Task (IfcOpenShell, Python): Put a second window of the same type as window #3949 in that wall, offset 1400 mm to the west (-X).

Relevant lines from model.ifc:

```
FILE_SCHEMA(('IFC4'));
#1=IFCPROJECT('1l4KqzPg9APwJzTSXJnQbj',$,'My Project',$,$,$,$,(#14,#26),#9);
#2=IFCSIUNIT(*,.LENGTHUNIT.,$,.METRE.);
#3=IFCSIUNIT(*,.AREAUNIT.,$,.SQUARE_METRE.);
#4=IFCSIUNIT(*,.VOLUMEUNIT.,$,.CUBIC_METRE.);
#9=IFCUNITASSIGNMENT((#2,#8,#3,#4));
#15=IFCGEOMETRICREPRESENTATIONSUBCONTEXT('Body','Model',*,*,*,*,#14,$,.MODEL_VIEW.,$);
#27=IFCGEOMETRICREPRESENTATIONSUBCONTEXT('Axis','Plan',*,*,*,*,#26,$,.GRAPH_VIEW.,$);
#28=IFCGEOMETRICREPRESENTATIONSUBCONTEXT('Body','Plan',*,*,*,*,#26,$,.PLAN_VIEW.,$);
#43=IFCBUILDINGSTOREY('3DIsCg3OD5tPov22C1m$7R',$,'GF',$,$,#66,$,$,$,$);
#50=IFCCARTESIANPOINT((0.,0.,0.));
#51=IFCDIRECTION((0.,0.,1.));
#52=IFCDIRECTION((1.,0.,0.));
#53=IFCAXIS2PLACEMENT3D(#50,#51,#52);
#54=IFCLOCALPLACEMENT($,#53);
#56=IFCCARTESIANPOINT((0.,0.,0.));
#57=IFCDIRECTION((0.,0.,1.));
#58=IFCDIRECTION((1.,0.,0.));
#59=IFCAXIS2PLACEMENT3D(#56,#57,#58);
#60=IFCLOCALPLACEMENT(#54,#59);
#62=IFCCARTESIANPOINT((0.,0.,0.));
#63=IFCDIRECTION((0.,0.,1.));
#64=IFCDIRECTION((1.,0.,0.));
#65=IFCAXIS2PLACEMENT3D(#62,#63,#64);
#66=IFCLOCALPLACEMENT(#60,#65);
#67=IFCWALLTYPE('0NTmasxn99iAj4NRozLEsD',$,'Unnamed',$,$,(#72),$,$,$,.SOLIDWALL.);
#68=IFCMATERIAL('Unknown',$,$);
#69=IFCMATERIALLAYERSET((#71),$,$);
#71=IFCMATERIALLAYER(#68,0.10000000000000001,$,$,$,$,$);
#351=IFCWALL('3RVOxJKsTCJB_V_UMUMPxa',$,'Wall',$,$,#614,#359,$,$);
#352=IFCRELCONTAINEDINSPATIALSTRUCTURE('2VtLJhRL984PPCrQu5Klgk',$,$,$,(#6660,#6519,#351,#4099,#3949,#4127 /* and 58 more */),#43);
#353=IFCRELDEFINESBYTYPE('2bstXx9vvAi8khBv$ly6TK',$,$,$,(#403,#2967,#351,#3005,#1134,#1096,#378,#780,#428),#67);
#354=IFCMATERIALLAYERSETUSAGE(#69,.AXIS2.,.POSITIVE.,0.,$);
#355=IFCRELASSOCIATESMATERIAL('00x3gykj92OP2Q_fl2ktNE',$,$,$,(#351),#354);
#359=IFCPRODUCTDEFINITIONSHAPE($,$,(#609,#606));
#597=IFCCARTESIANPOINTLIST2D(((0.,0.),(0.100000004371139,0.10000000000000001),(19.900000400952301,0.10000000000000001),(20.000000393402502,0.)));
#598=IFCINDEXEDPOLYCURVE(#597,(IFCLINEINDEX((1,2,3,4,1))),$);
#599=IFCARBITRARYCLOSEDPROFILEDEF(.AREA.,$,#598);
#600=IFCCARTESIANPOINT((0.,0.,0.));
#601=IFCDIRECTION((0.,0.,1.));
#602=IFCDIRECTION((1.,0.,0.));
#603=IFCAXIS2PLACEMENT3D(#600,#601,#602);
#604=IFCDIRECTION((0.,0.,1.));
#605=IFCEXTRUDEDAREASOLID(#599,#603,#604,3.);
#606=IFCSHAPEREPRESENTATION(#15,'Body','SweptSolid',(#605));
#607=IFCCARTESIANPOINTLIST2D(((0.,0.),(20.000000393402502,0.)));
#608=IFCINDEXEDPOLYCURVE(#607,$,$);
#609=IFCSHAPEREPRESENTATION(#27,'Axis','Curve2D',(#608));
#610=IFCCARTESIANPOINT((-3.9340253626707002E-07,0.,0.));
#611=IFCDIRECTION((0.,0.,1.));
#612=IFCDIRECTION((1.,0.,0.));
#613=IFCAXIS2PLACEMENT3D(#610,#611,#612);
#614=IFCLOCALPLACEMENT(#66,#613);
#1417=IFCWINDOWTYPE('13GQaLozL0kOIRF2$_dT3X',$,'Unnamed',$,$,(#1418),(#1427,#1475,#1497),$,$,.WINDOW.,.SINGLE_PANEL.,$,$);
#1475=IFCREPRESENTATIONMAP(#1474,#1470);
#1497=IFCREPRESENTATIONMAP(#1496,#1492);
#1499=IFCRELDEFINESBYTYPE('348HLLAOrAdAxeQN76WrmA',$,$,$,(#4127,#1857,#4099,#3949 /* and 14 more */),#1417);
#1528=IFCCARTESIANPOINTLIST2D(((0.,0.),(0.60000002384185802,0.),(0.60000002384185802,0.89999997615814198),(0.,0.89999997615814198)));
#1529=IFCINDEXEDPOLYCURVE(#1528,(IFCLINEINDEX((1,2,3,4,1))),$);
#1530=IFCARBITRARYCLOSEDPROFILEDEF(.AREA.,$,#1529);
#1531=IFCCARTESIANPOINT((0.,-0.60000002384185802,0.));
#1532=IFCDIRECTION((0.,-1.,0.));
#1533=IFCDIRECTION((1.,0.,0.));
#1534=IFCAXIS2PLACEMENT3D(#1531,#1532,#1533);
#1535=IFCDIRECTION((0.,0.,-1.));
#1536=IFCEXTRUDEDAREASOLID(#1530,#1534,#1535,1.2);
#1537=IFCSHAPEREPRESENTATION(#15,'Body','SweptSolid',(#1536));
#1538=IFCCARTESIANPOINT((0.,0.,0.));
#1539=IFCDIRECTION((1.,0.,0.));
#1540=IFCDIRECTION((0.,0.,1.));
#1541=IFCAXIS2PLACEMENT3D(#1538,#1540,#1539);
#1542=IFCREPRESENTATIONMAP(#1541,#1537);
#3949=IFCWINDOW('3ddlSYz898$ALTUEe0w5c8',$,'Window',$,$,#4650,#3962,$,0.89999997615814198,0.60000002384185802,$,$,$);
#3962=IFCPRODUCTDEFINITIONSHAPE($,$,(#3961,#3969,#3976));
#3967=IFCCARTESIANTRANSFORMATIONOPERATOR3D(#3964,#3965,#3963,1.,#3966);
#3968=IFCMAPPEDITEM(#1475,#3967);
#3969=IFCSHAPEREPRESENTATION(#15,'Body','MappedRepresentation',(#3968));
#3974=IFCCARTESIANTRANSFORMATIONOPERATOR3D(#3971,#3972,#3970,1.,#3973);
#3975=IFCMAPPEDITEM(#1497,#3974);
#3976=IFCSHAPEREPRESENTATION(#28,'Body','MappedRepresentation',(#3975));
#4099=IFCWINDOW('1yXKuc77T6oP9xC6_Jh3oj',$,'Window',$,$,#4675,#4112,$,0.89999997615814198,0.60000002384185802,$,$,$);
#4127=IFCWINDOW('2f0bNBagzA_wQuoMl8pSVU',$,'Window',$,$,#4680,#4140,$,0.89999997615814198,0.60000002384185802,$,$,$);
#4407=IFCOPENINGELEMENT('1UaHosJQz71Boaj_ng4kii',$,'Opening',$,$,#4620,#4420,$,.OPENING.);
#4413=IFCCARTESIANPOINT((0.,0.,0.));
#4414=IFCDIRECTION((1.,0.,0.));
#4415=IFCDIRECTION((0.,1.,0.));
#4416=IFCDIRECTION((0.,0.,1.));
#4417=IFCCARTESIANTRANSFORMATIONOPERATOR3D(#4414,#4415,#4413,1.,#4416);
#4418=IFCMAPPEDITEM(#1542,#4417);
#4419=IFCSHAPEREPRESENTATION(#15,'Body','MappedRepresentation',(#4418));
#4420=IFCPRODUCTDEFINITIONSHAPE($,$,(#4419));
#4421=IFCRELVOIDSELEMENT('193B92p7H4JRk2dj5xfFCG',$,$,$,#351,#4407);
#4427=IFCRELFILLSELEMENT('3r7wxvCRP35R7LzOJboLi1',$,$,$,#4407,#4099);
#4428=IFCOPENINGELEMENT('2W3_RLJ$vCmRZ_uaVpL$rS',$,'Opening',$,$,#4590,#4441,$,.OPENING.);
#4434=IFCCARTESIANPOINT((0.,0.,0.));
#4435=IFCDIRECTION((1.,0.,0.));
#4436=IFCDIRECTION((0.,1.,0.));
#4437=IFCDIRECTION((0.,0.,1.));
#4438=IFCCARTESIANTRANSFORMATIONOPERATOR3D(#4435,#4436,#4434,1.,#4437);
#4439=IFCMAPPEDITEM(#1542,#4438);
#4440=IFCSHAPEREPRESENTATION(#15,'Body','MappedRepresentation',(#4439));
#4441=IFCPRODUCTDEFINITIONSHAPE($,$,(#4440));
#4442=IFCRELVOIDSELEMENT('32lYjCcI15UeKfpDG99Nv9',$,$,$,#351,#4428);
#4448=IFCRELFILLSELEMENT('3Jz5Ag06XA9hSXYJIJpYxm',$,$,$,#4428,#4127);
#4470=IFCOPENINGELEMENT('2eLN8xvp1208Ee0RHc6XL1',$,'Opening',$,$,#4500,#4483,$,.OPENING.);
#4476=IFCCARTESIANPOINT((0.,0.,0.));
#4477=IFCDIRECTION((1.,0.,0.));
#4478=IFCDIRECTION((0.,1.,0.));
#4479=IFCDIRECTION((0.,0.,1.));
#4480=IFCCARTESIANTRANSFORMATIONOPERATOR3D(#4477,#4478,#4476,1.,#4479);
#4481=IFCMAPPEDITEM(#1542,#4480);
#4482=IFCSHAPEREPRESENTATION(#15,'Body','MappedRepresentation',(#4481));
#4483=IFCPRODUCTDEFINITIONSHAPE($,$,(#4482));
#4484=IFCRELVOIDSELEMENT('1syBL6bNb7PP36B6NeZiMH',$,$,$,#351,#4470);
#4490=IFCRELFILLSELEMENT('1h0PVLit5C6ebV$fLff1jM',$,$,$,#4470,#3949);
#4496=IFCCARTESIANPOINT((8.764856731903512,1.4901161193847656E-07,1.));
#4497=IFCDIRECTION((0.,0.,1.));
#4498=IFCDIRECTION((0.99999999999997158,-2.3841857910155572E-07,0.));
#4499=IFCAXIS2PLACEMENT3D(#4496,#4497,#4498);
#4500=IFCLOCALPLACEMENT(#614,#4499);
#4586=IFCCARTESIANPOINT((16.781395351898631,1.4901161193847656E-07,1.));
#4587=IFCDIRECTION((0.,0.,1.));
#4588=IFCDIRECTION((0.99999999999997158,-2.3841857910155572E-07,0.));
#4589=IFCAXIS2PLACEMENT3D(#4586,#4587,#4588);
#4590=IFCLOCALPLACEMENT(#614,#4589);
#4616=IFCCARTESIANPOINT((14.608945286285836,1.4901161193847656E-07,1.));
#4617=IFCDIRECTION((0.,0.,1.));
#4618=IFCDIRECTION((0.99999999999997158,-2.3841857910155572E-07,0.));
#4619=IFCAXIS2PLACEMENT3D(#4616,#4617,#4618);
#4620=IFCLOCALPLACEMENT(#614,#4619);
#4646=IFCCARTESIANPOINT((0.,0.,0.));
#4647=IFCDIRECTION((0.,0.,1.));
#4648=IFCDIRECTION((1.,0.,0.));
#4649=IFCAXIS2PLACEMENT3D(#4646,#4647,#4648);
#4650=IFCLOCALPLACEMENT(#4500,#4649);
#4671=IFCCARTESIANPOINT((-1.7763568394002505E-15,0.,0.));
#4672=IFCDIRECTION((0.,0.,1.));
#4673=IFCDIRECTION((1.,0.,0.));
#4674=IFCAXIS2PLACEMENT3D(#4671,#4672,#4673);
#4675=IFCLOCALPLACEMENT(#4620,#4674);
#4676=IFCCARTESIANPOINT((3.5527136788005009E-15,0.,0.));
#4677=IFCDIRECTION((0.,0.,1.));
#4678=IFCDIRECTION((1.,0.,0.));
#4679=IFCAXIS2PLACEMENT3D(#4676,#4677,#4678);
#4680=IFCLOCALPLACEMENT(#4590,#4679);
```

```python
import ifcopenshell
import ifcopenshell.api.feature
import ifcopenshell.api.geometry
import ifcopenshell.api.root
import ifcopenshell.geom
import ifcopenshell.util.element
import ifcopenshell.util.placement
import ifcopenshell.util.shape
import ifcopenshell.util.unit

model = ifcopenshell.open("model.ifc")
unit_scale = ifcopenshell.util.unit.calculate_unit_scale(model)
settings = ifcopenshell.geom.settings()


def volume(element):
    """Net volume in cubic metres, openings subtracted."""
    shape = ifcopenshell.geom.create_shape(settings, element)
    return ifcopenshell.util.shape.get_volume(shape.geometry)


window = model.by_id(3949)
opening = window.FillsVoids[0].RelatingOpeningElement
wall = opening.VoidsElements[0].RelatingBuildingElement
before = volume(wall)
shift = ifcopenshell.util.placement.get_local_placement(wall.ObjectPlacement)[:3, 0] * -1.4 / unit_scale

# copy_class copies the void relationship, type, container and properties, but no geometry.
new_opening = ifcopenshell.api.root.copy_class(model, product=opening)
new_opening.Representation = ifcopenshell.util.element.copy_deep(
    model, opening.Representation, exclude=["IfcGeometricRepresentationContext", "IfcRepresentationMap"]
)
new_window = ifcopenshell.api.root.copy_class(model, product=window)
new_window.Representation = ifcopenshell.util.element.copy_deep(
    model, window.Representation, exclude=["IfcGeometricRepresentationContext", "IfcRepresentationMap"]
)
ifcopenshell.api.feature.add_filling(model, opening=new_opening, element=new_window)

for old, new in ((opening, new_opening), (window, new_window)):
    matrix = ifcopenshell.util.placement.get_local_placement(old.ObjectPlacement)
    matrix[:3, 3] += shift
    ifcopenshell.api.geometry.edit_object_placement(model, product=new, matrix=matrix, is_si=False)

after = volume(wall)

print(f"wall volume {before:.3f} -> {after:.3f} m3")

model.write("model_edited.ifc")
```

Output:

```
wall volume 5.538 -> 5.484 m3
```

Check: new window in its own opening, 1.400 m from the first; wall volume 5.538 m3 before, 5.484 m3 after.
